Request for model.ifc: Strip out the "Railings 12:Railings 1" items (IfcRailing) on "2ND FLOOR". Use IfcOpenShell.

First a look at what the model holds.

```python
import ifcopenshell
import ifcopenshell.util.element

model = ifcopenshell.open("model.ifc")
print(model.schema)
storey = next(s for s in model.by_type("IfcBuildingStorey") if s.Name == "2ND FLOOR")
railings = [e for e in ifcopenshell.util.element.get_decomposition(storey) if e.is_a("IfcRailing")]
seen = {}
for e in railings:
    element_type = ifcopenshell.util.element.get_type(e)
    name = element_type.Name if element_type not in (None, e) else None
    seen[name] = seen.get(name, 0) + 1
for name, count in sorted(seen.items(), key=str):
    print(count, "x", name)
```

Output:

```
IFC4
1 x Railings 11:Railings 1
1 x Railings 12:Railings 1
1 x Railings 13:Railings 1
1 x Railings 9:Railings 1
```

```python
import ifcopenshell
import ifcopenshell.api.root
import ifcopenshell.util.element

model = ifcopenshell.open("model.ifc")

storey = next(s for s in model.by_type("IfcBuildingStorey") if s.Name == "2ND FLOOR")
railings = [e for e in ifcopenshell.util.element.get_decomposition(storey) if e.is_a("IfcRailing")]
targets = [e for e in railings if (t := ifcopenshell.util.element.get_type(e)) not in (None, e) and t.Name == "Railings 12:Railings 1"]

for e in targets:
    ifcopenshell.api.root.remove_product(model, product=e)
print(len(targets), "removed")

model.write("model_edited.ifc")
```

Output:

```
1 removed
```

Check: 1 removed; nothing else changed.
